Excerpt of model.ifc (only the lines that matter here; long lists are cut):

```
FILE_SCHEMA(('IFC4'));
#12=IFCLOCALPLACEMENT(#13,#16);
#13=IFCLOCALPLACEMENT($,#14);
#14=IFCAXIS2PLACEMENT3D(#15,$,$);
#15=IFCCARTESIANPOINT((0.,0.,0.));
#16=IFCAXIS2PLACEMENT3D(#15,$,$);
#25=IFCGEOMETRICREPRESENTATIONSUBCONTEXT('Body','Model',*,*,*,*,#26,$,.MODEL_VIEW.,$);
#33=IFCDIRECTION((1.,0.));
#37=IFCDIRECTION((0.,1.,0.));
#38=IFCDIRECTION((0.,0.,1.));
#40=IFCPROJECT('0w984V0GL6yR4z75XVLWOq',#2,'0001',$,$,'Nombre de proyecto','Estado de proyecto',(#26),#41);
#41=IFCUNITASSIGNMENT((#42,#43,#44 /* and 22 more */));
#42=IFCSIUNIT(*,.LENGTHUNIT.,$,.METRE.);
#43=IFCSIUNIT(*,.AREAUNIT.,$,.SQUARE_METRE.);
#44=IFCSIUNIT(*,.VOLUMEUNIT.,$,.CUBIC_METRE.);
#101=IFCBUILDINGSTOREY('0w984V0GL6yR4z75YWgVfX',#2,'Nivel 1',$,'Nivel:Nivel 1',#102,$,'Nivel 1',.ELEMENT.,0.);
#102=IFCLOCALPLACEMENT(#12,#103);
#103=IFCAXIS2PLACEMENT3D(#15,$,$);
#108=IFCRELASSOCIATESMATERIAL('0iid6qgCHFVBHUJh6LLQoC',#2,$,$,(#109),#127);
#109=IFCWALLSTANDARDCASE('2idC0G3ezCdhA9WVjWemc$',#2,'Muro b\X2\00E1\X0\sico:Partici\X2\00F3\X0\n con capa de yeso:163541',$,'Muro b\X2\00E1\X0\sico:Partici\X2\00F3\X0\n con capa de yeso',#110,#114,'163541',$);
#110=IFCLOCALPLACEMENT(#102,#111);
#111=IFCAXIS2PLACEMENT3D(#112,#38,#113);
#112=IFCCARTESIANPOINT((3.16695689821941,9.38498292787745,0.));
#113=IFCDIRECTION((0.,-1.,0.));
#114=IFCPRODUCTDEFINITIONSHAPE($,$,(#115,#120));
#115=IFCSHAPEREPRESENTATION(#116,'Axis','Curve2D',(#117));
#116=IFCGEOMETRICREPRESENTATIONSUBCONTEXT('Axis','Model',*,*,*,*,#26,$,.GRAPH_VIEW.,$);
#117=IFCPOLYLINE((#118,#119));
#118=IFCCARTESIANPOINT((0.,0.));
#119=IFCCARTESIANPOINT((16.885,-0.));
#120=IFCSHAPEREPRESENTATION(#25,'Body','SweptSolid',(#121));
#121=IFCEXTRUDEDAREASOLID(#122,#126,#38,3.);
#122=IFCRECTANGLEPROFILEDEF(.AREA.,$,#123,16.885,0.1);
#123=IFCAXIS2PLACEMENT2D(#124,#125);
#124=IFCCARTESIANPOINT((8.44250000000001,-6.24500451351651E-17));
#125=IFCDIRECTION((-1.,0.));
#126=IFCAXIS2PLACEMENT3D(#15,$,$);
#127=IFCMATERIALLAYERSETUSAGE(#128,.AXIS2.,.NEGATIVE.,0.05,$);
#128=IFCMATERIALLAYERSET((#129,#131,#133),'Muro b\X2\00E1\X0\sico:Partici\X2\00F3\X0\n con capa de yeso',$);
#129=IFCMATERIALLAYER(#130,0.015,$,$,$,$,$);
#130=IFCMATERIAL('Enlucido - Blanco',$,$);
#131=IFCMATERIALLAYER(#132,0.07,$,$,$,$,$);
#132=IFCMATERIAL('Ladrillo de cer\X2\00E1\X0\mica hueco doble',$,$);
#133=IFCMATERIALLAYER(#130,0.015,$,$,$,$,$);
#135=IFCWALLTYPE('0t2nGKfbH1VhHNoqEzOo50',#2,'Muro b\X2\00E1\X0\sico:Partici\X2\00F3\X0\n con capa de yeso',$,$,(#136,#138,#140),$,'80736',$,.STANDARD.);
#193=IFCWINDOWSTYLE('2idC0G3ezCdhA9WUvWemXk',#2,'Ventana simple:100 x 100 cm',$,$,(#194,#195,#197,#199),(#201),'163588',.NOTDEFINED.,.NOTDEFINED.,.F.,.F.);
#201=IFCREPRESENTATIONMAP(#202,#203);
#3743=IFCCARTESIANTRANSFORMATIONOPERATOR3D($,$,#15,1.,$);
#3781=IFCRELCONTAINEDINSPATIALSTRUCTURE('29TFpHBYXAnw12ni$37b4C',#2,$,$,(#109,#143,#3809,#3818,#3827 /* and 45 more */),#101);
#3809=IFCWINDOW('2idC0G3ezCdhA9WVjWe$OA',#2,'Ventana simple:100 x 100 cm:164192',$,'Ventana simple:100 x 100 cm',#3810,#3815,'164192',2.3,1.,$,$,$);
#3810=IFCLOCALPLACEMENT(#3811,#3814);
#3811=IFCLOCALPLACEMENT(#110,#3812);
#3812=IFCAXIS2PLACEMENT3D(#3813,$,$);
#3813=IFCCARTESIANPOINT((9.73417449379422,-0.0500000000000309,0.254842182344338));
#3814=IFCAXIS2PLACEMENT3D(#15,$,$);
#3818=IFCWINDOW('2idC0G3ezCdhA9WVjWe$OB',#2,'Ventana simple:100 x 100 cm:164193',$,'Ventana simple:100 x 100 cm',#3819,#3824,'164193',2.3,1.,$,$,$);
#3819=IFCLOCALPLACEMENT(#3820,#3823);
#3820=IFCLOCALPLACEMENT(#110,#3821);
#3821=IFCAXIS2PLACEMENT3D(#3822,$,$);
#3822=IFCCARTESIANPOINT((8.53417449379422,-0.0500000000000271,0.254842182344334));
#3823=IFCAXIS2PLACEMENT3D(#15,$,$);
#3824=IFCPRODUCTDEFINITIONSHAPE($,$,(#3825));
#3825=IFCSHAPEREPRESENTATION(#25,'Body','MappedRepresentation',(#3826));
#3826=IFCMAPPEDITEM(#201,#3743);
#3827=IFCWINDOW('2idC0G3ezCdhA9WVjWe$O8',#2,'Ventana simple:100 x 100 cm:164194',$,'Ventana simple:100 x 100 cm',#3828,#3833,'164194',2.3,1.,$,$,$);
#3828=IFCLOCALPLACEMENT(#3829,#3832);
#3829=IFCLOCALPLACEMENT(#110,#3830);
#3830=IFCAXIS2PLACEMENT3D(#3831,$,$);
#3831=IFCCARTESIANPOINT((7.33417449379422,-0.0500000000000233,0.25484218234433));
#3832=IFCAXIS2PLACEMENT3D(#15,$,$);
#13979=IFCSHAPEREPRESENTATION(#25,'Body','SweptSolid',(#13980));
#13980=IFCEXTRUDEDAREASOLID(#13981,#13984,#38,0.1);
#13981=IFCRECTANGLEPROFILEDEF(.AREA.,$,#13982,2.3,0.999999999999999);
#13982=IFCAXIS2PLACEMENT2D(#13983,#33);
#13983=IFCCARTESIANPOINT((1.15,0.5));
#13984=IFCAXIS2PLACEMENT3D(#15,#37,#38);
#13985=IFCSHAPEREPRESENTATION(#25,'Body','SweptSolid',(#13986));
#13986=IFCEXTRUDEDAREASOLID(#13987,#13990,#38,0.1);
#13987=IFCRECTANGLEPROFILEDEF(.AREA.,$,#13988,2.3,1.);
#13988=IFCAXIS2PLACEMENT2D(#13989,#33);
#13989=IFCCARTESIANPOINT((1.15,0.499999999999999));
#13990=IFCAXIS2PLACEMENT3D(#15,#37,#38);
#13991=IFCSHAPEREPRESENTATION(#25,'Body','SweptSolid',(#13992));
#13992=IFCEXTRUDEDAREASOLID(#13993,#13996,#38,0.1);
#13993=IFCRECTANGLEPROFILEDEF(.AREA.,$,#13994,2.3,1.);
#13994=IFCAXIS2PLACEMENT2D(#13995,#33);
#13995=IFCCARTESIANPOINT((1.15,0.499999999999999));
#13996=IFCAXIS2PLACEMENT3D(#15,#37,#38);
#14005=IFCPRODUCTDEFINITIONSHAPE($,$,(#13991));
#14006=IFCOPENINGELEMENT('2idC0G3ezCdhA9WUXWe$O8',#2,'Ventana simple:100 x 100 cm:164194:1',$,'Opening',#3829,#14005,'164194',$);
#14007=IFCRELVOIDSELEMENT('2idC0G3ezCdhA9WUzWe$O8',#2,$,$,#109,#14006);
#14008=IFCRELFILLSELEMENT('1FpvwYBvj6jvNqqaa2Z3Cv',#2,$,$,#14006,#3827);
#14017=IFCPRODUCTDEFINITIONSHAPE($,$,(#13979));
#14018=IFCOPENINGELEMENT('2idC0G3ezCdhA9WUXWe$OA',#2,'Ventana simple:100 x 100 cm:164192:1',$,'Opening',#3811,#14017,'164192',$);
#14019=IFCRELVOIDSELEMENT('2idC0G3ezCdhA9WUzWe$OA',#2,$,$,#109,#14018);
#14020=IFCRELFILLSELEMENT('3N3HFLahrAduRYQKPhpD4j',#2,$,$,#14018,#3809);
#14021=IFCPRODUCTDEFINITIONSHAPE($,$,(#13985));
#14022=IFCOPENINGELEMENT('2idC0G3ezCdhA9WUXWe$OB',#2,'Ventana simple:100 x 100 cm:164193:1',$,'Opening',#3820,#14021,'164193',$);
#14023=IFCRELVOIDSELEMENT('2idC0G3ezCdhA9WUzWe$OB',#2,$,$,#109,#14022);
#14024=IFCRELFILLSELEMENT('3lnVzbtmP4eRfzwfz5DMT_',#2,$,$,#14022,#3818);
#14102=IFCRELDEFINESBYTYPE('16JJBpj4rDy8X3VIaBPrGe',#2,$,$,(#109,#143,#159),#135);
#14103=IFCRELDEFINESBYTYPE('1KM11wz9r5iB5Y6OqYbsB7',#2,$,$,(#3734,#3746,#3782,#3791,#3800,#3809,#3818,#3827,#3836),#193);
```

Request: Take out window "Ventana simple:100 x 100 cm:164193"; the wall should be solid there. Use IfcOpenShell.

```python
import ifcopenshell
import ifcopenshell.api.feature
import ifcopenshell.api.root
import ifcopenshell.geom
import ifcopenshell.util.shape

model = ifcopenshell.open("model.ifc")
settings = ifcopenshell.geom.settings()


def volume(element):
    """Net volume in cubic metres, openings subtracted."""
    shape = ifcopenshell.geom.create_shape(settings, element)
    return ifcopenshell.util.shape.get_volume(shape.geometry)


window = model.by_guid("2idC0G3ezCdhA9WVjWe$OB")
opening = window.FillsVoids[0].RelatingOpeningElement
wall = opening.VoidsElements[0].RelatingBuildingElement
before = volume(wall)

ifcopenshell.api.root.remove_product(model, product=window)
ifcopenshell.api.feature.remove_feature(model, feature=opening)

after = volume(wall)

print(f"wall volume {before:.3f} -> {after:.3f} m3")

model.write("model_v2.ifc")
```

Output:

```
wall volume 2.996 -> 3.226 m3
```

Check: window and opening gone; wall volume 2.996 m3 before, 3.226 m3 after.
